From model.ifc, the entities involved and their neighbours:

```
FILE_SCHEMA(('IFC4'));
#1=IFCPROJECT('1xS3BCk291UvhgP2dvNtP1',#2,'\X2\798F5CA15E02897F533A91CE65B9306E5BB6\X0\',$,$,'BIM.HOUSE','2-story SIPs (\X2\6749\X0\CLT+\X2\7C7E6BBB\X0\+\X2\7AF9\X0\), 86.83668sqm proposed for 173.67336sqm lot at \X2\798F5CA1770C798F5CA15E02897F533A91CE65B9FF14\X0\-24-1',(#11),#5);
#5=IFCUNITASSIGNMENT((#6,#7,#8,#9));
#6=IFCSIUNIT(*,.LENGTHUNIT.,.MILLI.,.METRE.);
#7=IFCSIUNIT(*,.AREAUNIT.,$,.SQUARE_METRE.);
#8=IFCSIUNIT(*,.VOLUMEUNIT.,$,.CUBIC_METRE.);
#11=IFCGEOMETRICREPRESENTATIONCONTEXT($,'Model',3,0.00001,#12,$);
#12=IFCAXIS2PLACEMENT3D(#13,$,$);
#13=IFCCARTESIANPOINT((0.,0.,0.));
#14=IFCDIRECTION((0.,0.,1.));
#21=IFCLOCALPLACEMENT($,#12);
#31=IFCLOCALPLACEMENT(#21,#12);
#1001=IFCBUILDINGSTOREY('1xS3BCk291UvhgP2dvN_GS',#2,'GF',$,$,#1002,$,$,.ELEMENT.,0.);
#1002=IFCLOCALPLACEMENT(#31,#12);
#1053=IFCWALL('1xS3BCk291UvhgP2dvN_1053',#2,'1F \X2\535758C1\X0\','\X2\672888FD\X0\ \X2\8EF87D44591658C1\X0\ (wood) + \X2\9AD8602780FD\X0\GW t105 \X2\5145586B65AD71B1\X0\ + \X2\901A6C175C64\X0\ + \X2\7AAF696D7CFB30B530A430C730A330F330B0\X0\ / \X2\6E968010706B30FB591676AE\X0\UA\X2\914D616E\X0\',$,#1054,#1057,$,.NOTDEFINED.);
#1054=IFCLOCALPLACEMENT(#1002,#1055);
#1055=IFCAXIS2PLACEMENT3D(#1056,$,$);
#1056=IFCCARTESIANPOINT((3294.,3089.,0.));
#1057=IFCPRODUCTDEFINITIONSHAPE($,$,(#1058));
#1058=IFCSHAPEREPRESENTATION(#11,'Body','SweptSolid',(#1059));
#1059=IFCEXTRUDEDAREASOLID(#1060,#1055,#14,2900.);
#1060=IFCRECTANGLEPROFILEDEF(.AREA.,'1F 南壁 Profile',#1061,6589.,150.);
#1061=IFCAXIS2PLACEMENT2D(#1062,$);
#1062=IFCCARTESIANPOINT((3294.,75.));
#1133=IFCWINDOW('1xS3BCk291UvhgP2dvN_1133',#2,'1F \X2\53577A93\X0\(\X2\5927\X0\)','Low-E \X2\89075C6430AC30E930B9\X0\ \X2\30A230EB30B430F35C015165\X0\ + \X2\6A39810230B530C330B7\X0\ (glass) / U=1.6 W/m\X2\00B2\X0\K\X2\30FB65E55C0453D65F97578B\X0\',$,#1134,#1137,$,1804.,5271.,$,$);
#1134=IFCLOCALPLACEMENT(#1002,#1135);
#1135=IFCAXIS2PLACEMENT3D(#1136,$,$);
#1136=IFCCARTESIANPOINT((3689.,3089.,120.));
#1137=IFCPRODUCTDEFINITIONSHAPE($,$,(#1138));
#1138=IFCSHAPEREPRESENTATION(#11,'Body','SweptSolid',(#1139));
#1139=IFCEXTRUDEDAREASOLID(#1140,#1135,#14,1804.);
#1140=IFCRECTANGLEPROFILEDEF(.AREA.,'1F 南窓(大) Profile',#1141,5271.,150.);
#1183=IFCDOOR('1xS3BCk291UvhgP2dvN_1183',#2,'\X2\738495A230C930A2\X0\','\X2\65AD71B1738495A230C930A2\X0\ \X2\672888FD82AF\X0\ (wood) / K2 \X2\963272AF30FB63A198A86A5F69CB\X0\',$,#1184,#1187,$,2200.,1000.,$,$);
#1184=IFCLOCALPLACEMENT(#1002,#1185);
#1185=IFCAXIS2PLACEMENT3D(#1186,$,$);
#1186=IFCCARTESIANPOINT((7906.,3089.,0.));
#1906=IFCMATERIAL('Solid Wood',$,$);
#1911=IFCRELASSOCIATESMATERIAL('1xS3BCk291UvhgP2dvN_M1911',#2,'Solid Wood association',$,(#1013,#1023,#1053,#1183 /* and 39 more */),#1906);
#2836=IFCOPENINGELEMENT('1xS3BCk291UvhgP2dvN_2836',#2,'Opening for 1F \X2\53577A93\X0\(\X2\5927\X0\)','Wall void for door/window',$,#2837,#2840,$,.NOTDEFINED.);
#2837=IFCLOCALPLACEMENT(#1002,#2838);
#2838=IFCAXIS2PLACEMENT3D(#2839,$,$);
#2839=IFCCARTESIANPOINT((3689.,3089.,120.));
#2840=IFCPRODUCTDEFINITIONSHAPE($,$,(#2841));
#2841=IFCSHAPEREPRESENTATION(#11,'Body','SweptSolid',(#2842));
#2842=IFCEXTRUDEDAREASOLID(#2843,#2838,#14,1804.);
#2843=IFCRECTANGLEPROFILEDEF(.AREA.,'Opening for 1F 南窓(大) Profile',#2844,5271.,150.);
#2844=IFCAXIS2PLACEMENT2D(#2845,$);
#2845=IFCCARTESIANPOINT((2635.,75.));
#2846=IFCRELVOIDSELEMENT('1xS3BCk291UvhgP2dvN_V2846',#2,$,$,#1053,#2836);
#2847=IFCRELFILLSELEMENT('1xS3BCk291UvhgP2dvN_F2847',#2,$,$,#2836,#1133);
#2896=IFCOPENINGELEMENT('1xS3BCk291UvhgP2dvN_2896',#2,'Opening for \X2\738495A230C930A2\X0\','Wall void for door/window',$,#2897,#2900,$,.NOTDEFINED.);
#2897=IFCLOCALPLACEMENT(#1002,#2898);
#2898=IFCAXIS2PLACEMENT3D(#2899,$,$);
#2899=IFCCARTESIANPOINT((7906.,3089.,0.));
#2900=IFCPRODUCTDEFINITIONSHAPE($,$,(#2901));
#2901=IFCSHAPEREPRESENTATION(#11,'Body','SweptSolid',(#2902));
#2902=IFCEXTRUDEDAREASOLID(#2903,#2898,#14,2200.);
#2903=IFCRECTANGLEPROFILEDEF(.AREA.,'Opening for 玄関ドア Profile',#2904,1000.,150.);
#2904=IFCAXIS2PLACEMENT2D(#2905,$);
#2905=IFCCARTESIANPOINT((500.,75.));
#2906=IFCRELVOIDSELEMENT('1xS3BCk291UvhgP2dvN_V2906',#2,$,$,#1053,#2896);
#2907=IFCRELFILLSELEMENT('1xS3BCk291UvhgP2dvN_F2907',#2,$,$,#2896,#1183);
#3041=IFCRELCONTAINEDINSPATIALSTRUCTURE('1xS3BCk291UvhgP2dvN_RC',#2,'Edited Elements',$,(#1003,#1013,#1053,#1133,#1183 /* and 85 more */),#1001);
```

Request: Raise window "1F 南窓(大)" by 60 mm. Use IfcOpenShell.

```python
import numpy as np
import ifcopenshell
import ifcopenshell.api.geometry
import ifcopenshell.util.placement
import ifcopenshell.util.unit

model = ifcopenshell.open("model.ifc")
unit_scale = ifcopenshell.util.unit.calculate_unit_scale(model)

window = model.by_guid("1xS3BCk291UvhgP2dvN_1133")
opening = window.FillsVoids[0].RelatingOpeningElement
dz = 0.06 / unit_scale

shift = np.array([0.0, 0.0, dz])
# The window is not placed relative to its opening, so move both.
for product in (opening, window):
    matrix = ifcopenshell.util.placement.get_local_placement(product.ObjectPlacement)
    matrix[:3, 3] += shift
    ifcopenshell.api.geometry.edit_object_placement(model, product=product, matrix=matrix, is_si=False)

print(f"moved by {dz * unit_scale:+.3f} m")

model.write("model_edited.ifc")
```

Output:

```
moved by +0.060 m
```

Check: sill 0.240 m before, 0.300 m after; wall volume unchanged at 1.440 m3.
